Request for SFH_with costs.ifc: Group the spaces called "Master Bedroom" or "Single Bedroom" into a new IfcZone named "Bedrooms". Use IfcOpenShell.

First a look at what the model holds.

```python
import ifcopenshell

model = ifcopenshell.open("SFH_with costs.ifc")
print(model.schema)
seen = {}
for space in model.by_type("IfcSpace"):
    seen[space.LongName] = seen.get(space.LongName, 0) + 1
for name, count in sorted(seen.items(), key=str):
    print(count, "x", name)
print("zones:", [z.Name for z in model.by_type("IfcZone")][:20])
```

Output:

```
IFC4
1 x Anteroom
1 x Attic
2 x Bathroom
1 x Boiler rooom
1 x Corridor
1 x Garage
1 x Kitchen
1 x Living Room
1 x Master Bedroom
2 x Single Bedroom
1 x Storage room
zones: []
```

```python
import ifcopenshell
import ifcopenshell.api.group
import ifcopenshell.api.root

model = ifcopenshell.open("SFH_with costs.ifc")

names = {"Master Bedroom", "Single Bedroom"}
spaces = [s for s in model.by_type("IfcSpace") if s.LongName in names]

zone = ifcopenshell.api.root.create_entity(model, ifc_class="IfcZone", name="Bedrooms")
ifcopenshell.api.group.assign_group(model, products=spaces, group=zone)
print(len(spaces), "spaces in", zone.Name)

model.write("SFH_with costs_rev.ifc")
```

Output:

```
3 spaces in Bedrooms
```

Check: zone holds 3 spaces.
